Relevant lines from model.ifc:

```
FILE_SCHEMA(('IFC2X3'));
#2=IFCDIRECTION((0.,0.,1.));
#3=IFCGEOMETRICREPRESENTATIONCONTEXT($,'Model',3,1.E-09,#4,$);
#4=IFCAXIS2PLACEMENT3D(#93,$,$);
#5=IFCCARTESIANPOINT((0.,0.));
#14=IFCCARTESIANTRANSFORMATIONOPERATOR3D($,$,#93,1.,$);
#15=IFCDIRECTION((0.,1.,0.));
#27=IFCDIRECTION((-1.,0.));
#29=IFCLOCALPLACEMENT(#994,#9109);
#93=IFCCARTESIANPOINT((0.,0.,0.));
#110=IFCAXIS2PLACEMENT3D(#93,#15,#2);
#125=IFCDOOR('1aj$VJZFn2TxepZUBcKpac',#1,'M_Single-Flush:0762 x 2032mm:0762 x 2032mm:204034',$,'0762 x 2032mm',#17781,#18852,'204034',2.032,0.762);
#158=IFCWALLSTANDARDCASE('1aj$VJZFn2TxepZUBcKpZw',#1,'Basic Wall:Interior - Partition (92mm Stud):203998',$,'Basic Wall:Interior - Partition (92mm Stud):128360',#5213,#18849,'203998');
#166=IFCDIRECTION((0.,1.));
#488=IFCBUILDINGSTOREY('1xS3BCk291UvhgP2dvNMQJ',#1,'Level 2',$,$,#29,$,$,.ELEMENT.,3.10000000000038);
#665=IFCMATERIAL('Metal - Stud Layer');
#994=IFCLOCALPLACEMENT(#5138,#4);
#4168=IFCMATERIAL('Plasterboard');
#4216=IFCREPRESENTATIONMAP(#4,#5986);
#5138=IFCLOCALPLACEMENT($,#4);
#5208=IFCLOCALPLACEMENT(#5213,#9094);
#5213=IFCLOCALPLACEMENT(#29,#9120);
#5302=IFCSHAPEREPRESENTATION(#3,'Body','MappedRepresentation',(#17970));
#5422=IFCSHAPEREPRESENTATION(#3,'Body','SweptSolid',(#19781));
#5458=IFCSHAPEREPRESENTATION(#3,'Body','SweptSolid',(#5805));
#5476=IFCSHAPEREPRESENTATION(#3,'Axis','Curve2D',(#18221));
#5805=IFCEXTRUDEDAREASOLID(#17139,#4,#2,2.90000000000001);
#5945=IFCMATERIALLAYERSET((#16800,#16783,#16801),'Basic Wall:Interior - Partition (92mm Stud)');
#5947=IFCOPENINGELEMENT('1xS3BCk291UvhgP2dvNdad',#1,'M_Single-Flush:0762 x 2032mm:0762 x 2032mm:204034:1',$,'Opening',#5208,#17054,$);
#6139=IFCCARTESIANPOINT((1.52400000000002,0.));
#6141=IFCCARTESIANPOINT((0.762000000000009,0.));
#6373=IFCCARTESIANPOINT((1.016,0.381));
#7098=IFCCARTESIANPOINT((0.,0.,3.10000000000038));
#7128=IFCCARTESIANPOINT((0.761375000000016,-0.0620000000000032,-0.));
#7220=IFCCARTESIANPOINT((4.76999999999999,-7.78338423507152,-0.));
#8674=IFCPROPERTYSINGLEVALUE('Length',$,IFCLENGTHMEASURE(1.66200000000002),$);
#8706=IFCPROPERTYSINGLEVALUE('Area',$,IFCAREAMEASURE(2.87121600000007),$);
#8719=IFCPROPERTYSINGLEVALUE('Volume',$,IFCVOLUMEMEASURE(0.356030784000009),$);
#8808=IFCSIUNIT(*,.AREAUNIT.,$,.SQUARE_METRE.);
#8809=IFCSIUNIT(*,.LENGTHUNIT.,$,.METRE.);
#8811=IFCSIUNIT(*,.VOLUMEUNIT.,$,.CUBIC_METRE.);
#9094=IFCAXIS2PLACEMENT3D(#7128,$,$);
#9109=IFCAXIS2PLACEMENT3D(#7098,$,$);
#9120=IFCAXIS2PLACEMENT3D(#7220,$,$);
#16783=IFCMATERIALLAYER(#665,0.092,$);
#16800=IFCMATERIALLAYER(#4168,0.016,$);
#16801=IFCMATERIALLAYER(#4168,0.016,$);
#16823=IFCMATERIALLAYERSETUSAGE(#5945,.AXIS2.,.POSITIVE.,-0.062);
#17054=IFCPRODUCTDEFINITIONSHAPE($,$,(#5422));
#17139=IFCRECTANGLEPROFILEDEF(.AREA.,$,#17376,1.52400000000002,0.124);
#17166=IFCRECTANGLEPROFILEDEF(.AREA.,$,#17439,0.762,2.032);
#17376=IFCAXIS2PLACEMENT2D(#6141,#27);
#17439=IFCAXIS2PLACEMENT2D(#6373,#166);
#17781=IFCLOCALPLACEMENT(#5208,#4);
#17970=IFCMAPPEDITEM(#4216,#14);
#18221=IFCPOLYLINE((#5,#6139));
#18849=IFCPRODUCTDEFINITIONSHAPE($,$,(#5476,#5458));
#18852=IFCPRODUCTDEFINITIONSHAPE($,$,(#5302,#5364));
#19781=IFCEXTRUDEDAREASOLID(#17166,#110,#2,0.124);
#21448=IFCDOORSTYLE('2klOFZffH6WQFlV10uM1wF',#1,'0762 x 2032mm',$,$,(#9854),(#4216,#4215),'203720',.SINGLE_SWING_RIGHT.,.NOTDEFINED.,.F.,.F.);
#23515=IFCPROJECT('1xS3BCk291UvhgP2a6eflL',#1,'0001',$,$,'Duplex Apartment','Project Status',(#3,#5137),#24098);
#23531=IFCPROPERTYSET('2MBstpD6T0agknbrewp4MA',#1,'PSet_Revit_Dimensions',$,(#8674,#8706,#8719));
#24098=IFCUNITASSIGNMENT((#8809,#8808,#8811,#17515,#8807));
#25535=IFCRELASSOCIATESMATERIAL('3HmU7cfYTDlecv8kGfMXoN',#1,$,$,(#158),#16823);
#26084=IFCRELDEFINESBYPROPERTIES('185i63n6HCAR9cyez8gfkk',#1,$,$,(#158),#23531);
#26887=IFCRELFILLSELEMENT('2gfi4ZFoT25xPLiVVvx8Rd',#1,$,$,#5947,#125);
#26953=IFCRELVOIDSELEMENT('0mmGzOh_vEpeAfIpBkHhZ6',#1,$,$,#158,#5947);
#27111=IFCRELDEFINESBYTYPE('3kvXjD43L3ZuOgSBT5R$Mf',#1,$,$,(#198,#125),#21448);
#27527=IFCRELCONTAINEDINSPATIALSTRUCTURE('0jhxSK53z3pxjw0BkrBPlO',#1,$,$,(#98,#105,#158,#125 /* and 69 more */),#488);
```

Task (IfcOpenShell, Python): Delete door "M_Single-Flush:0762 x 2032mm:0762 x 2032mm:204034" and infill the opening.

```python
import ifcopenshell
import ifcopenshell.api.feature
import ifcopenshell.api.pset
import ifcopenshell.api.root
import ifcopenshell.geom
import ifcopenshell.util.element
import ifcopenshell.util.shape
import ifcopenshell.util.unit

model = ifcopenshell.open("model.ifc")
area_scale = ifcopenshell.util.unit.calculate_unit_scale(model, "AREAUNIT")
volume_scale = ifcopenshell.util.unit.calculate_unit_scale(model, "VOLUMEUNIT")
settings = ifcopenshell.geom.settings()


def volume(element):
    """Net volume in cubic metres, openings subtracted."""
    shape = ifcopenshell.geom.create_shape(settings, element)
    return ifcopenshell.util.shape.get_volume(shape.geometry)


door = model.by_guid("1aj$VJZFn2TxepZUBcKpac")
opening = door.FillsVoids[0].RelatingOpeningElement
wall = opening.VoidsElements[0].RelatingBuildingElement
before = volume(wall)

ifcopenshell.api.root.remove_product(model, product=door)
ifcopenshell.api.feature.remove_feature(model, feature=opening)

after = volume(wall)
thickness = 0.124  # wall thickness in metres

# Update the wall's stored quantities.
pset = model.by_id(ifcopenshell.util.element.get_pset(wall, "PSet_Revit_Dimensions", should_inherit=False)["id"])
ifcopenshell.api.pset.edit_pset(model, pset=pset, properties={
    "Area": model.create_entity("IfcAreaMeasure", after / thickness / area_scale),
    "Volume": model.create_entity("IfcVolumeMeasure", after / volume_scale),
})

print(f"wall volume {before:.3f} -> {after:.3f} m3")

model.write("model_updated.ifc")
```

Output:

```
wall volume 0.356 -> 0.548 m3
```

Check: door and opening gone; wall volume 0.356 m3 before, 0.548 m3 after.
